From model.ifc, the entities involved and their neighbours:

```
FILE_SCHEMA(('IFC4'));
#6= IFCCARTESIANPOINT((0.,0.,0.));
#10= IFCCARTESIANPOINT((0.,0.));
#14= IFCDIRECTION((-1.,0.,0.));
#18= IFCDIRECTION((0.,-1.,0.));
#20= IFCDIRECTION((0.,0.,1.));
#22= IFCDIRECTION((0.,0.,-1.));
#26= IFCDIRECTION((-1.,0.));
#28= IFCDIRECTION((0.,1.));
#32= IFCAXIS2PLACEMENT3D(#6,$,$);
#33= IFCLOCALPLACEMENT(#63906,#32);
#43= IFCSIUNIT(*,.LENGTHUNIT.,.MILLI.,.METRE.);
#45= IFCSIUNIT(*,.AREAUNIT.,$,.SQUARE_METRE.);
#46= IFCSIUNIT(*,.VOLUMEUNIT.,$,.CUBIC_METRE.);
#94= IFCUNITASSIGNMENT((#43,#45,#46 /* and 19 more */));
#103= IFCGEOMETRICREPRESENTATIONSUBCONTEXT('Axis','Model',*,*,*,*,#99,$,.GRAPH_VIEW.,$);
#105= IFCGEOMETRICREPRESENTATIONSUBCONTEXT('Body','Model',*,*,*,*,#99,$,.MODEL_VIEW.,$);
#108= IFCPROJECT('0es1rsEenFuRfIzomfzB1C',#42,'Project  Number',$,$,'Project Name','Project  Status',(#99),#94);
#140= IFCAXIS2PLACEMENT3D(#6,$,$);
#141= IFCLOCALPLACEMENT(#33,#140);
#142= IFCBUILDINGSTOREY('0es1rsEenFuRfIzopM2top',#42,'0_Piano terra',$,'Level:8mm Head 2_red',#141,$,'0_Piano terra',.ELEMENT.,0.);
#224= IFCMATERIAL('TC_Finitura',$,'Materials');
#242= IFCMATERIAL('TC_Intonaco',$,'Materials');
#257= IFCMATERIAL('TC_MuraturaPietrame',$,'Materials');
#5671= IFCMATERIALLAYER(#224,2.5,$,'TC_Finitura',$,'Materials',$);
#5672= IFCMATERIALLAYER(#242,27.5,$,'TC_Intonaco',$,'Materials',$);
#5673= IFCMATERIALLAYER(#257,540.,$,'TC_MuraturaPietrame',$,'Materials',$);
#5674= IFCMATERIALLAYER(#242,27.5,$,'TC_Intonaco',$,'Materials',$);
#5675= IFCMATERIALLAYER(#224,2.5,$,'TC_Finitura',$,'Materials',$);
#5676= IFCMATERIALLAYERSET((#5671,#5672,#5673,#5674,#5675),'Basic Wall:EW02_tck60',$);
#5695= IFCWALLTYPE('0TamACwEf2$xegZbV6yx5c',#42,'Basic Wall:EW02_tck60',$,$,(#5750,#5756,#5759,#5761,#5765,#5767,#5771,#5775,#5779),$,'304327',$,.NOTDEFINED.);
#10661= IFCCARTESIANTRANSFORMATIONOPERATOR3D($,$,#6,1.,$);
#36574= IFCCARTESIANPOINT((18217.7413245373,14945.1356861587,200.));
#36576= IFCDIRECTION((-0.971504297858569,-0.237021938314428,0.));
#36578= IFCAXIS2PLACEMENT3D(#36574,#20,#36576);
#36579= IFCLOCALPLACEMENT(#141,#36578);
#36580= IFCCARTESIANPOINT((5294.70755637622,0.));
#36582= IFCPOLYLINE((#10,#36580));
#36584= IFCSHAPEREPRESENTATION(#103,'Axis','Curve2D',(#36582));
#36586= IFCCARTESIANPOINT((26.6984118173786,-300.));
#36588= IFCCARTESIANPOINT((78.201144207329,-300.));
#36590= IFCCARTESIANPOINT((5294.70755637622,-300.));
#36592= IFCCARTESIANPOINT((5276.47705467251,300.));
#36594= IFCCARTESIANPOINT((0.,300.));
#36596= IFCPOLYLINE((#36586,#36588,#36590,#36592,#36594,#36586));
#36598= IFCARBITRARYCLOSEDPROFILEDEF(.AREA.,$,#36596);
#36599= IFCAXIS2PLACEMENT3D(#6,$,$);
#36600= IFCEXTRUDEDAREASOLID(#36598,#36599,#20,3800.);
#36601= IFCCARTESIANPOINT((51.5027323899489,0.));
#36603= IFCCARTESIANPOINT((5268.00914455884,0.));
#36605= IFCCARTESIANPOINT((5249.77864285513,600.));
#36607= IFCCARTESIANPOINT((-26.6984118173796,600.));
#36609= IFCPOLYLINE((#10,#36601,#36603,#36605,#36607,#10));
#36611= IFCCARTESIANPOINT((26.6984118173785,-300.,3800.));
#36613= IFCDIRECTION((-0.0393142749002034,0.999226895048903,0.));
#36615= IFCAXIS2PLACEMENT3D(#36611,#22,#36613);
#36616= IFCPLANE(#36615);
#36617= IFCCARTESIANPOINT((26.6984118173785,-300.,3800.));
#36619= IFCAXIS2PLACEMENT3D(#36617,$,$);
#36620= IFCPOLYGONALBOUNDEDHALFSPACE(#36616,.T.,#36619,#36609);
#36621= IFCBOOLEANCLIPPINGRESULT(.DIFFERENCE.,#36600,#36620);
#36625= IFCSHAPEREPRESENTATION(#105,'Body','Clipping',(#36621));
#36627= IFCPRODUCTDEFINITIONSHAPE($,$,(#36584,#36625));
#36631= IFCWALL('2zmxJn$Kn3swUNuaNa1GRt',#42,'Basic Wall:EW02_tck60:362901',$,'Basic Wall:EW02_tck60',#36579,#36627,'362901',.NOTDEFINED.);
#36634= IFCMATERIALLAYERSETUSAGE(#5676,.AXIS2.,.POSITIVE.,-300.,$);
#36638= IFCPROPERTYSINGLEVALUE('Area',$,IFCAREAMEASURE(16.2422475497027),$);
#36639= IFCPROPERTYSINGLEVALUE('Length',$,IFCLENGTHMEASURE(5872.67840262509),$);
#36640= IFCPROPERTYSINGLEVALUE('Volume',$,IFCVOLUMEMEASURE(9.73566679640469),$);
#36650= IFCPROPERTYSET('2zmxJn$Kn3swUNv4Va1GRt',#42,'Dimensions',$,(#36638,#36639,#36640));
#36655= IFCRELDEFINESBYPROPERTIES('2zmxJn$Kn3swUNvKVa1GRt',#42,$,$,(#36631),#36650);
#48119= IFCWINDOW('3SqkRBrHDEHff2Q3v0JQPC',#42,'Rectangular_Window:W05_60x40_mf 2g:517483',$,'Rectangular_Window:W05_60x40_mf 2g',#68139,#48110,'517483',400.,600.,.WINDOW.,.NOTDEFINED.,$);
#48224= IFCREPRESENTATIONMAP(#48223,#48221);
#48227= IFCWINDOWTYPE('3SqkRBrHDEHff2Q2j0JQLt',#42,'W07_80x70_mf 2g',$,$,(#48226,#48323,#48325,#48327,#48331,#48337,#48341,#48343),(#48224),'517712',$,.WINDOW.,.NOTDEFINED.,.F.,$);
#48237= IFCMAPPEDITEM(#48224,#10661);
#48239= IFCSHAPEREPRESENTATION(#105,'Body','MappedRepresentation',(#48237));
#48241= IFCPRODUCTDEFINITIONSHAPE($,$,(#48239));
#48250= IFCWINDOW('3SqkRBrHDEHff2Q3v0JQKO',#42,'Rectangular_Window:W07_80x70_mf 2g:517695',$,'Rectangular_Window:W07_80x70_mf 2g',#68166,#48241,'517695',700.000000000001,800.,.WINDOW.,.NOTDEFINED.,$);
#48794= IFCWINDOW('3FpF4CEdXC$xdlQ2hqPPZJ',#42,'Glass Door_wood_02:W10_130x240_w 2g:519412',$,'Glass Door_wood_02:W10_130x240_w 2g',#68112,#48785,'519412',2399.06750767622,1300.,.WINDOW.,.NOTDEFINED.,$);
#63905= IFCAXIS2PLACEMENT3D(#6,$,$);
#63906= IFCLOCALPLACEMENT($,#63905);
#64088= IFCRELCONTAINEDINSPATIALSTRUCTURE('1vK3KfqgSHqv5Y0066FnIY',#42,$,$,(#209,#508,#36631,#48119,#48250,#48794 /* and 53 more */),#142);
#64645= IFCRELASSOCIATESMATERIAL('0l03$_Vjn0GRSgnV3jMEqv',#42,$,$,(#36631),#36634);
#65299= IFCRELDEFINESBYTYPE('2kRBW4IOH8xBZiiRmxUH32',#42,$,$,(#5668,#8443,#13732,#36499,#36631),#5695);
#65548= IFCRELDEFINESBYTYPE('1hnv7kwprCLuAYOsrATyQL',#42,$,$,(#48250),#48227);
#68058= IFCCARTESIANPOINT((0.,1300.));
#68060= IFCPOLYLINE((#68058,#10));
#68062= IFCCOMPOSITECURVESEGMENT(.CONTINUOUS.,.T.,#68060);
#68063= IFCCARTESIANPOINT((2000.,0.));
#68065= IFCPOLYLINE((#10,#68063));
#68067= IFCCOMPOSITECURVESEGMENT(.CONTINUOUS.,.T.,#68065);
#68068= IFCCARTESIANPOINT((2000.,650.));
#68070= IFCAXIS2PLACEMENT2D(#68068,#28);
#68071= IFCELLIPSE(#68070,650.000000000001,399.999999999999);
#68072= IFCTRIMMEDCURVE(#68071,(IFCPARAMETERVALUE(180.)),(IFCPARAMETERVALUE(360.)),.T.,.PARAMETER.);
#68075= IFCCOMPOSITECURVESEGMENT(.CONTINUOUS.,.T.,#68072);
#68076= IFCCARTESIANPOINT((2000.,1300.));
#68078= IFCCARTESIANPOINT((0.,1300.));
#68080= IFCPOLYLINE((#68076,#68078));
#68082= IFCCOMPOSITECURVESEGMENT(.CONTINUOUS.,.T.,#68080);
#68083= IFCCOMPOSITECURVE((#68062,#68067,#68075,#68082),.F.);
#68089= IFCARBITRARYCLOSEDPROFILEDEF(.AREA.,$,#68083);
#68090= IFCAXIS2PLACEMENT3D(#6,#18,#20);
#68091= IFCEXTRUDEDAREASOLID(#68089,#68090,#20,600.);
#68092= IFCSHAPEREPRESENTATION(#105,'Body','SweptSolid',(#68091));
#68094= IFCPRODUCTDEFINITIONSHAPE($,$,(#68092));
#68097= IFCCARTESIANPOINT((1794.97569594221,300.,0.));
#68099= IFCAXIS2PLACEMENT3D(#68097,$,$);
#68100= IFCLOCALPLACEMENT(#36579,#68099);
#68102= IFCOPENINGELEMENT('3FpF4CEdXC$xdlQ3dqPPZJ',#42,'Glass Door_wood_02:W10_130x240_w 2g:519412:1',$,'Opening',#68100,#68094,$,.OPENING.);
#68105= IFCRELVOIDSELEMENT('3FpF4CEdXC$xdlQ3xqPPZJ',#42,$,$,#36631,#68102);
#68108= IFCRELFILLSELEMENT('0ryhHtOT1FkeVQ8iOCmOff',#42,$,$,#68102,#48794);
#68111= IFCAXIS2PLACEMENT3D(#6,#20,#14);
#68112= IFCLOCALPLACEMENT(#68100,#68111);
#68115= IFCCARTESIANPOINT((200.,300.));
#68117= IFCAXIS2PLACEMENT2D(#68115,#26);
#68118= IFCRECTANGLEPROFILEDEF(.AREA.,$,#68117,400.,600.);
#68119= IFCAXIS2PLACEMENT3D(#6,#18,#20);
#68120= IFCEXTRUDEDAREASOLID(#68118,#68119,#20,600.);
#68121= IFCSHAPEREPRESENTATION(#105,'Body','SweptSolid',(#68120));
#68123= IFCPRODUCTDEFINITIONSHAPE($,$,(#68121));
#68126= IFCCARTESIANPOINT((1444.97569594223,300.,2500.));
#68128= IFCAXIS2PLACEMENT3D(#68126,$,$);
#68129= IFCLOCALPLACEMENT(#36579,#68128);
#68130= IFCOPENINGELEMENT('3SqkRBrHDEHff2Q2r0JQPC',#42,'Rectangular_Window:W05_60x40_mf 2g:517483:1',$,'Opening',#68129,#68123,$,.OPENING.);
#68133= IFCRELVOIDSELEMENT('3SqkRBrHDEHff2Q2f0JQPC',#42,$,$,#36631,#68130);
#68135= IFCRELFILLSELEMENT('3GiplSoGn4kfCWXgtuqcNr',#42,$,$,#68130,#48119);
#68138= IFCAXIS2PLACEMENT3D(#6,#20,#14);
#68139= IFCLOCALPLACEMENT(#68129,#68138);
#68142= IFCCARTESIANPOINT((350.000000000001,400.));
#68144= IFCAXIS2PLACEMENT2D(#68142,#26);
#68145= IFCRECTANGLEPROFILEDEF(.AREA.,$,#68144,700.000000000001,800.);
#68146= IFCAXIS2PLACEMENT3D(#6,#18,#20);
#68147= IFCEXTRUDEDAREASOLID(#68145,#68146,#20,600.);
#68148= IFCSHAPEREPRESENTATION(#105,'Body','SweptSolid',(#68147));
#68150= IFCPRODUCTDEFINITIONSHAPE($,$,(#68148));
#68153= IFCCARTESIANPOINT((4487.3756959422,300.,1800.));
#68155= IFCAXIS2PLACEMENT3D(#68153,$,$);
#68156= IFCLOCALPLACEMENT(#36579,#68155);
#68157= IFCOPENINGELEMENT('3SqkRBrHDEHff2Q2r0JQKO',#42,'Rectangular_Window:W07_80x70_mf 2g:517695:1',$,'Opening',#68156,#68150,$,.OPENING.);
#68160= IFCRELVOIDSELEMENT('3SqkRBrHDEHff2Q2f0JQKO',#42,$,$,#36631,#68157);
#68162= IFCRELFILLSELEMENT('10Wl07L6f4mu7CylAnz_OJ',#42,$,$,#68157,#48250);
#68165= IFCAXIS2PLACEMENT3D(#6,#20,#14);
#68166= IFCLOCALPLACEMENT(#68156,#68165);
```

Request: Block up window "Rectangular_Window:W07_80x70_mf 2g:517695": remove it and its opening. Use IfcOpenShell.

```python
import ifcopenshell
import ifcopenshell.api.feature
import ifcopenshell.api.pset
import ifcopenshell.api.root
import ifcopenshell.geom
import ifcopenshell.util.element
import ifcopenshell.util.shape
import ifcopenshell.util.unit

model = ifcopenshell.open("model.ifc")
area_scale = ifcopenshell.util.unit.calculate_unit_scale(model, "AREAUNIT")
volume_scale = ifcopenshell.util.unit.calculate_unit_scale(model, "VOLUMEUNIT")
settings = ifcopenshell.geom.settings()


def volume(element):
    """Net volume in cubic metres, openings subtracted."""
    shape = ifcopenshell.geom.create_shape(settings, element)
    return ifcopenshell.util.shape.get_volume(shape.geometry)


window = model.by_guid("3SqkRBrHDEHff2Q3v0JQKO")
opening = window.FillsVoids[0].RelatingOpeningElement
wall = opening.VoidsElements[0].RelatingBuildingElement
before = volume(wall)

ifcopenshell.api.root.remove_product(model, product=window)
ifcopenshell.api.feature.remove_feature(model, feature=opening)

after = volume(wall)
thickness = 0.6  # wall thickness in metres

# Update the wall's stored quantities.
pset = model.by_id(ifcopenshell.util.element.get_pset(wall, "Dimensions", should_inherit=False)["id"])
ifcopenshell.api.pset.edit_pset(model, pset=pset, properties={
    "Area": model.create_entity("IfcAreaMeasure", after / thickness / area_scale),
    "Volume": model.create_entity("IfcVolumeMeasure", after / volume_scale),
})

print(f"wall volume {before:.3f} -> {after:.3f} m3")

model.write("model_updated.ifc")
```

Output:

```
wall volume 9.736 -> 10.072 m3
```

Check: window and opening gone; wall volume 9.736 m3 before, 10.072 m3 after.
